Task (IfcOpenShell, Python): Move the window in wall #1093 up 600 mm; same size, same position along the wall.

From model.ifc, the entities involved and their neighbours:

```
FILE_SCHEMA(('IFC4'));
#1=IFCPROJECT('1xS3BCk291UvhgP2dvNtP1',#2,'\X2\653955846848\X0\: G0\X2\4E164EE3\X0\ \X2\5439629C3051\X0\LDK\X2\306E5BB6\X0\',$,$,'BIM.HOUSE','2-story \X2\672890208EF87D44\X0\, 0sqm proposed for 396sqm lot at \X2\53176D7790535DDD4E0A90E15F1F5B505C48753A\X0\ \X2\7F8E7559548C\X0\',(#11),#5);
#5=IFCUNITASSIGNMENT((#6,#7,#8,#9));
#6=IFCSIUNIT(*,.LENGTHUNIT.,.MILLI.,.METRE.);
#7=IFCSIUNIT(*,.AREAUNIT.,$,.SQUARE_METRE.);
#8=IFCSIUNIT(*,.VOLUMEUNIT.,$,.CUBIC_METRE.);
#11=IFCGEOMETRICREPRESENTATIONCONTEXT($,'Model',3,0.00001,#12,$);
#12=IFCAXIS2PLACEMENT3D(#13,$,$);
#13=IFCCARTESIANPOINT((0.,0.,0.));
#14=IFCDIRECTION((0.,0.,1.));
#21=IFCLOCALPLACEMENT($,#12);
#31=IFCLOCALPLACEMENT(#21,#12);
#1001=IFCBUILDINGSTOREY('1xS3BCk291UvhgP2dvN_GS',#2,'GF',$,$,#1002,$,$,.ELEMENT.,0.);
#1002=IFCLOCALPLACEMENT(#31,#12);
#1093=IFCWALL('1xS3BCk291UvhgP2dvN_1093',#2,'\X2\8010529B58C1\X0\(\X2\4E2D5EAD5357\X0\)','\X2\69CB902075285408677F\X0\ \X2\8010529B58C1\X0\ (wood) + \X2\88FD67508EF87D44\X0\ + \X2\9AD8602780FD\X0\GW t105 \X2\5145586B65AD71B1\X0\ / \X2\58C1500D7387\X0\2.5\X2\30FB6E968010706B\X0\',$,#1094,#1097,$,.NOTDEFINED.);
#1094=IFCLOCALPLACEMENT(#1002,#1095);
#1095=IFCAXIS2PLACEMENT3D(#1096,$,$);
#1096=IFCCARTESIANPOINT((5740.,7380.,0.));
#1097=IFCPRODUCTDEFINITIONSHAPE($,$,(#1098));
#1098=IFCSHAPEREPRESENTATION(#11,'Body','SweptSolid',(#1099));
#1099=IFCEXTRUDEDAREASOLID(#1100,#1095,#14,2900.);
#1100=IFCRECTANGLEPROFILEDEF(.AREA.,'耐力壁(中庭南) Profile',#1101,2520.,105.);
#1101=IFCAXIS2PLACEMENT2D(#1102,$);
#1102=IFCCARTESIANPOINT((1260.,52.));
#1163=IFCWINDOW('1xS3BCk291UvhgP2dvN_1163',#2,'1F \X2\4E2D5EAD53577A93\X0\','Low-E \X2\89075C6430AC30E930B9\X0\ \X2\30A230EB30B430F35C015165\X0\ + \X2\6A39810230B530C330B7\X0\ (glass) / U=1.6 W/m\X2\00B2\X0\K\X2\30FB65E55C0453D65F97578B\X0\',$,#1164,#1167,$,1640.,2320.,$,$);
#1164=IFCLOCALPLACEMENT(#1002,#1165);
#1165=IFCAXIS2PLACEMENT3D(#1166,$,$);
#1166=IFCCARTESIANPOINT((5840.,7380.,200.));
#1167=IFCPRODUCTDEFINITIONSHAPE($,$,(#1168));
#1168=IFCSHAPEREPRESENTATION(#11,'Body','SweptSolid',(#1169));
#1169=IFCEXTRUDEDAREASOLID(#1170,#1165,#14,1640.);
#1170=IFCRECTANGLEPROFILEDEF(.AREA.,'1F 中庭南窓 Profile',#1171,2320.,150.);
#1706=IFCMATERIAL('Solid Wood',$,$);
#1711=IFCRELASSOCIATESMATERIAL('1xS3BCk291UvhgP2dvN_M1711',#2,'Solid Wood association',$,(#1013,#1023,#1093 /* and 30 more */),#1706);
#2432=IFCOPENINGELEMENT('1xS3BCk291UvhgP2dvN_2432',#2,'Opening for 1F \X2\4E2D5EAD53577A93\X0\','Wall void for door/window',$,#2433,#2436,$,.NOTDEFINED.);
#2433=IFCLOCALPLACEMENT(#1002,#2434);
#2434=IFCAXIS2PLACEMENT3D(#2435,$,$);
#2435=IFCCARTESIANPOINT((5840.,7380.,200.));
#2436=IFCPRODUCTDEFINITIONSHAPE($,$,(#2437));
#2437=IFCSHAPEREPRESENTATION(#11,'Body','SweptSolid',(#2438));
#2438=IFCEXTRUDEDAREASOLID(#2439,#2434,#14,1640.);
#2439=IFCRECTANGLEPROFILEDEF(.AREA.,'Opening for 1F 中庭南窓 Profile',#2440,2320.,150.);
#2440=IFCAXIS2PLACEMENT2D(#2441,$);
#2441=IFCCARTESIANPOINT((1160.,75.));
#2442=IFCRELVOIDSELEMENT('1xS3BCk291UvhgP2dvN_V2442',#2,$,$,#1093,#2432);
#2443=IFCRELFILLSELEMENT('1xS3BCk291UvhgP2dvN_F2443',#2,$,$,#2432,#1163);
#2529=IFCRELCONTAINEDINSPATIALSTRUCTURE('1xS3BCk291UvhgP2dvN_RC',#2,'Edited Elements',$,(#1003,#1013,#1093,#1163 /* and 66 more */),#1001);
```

```python
import numpy as np
import ifcopenshell
import ifcopenshell.api.geometry
import ifcopenshell.util.placement
import ifcopenshell.util.unit

model = ifcopenshell.open("model.ifc")
unit_scale = ifcopenshell.util.unit.calculate_unit_scale(model)

window = model.by_guid("1xS3BCk291UvhgP2dvN_1163")
opening = window.FillsVoids[0].RelatingOpeningElement
dz = 0.6 / unit_scale

shift = np.array([0.0, 0.0, dz])
# The window is not placed relative to its opening, so move both.
for product in (opening, window):
    matrix = ifcopenshell.util.placement.get_local_placement(product.ObjectPlacement)
    matrix[:3, 3] += shift
    ifcopenshell.api.geometry.edit_object_placement(model, product=product, matrix=matrix, is_si=False)

print(f"moved by {dz * unit_scale:+.3f} m")

model.write("model_rev.ifc")
```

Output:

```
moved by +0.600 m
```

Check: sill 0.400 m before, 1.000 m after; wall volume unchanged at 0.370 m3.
